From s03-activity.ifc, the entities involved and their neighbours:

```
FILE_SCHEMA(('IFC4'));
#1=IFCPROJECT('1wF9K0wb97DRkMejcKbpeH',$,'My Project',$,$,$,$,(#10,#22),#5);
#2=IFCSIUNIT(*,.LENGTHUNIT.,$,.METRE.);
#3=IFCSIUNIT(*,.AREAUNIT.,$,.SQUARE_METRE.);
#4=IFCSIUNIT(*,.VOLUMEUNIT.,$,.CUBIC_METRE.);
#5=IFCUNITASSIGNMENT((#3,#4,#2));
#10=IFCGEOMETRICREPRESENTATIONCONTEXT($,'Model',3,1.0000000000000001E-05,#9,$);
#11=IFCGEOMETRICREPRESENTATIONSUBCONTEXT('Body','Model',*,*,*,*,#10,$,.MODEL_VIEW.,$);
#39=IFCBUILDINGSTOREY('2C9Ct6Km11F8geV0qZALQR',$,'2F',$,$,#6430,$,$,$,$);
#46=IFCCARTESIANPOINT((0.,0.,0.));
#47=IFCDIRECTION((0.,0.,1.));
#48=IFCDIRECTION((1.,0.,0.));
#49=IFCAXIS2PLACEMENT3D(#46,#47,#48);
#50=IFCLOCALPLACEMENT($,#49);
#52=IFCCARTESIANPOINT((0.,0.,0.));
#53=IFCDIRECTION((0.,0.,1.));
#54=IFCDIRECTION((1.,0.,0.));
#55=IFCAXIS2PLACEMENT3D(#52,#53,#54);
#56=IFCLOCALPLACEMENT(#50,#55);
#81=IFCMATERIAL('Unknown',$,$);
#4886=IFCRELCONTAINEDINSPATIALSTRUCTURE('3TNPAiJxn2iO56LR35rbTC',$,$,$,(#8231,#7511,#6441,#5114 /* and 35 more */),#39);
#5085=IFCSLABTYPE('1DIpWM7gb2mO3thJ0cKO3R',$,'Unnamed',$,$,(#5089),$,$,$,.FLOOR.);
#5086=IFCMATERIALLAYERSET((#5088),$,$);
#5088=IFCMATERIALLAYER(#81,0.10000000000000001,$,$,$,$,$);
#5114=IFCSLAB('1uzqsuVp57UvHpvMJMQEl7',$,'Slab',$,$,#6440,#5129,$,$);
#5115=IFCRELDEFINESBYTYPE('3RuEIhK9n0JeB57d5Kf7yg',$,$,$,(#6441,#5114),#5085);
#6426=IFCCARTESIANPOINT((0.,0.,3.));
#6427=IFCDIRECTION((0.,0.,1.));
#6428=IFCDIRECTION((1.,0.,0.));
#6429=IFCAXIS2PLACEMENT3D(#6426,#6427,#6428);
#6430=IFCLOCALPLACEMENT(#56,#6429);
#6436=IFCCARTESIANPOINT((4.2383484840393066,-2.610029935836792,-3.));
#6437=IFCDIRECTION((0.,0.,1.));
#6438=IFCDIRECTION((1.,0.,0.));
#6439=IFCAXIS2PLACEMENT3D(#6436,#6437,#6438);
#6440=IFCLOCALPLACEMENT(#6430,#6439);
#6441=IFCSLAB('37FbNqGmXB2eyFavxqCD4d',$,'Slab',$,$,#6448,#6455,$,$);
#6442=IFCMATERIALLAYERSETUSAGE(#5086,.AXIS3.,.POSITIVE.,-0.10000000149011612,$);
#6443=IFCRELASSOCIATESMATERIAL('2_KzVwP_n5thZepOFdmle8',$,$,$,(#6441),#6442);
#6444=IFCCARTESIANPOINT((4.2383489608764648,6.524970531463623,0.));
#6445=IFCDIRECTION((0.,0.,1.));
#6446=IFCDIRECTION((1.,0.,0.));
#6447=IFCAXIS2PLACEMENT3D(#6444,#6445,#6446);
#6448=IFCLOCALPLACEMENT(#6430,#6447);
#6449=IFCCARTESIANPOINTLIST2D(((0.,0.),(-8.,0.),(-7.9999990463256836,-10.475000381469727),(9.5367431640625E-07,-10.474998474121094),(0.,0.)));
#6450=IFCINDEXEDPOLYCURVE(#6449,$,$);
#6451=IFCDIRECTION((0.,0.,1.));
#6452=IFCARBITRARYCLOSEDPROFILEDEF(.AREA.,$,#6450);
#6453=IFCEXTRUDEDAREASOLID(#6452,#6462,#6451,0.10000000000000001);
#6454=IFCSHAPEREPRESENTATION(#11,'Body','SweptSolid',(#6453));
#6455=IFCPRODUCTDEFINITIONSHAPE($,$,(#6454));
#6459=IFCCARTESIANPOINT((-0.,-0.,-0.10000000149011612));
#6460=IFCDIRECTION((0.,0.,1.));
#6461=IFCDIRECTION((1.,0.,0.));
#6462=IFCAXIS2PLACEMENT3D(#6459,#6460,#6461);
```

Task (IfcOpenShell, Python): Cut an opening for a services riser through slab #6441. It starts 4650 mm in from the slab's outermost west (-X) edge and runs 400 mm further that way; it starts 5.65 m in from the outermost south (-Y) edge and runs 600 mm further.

```python
import numpy as np
import ifcopenshell
import ifcopenshell.api.feature
import ifcopenshell.api.geometry
import ifcopenshell.api.root
import ifcopenshell.geom
import ifcopenshell.util.placement
import ifcopenshell.util.representation
import ifcopenshell.util.shape
import ifcopenshell.util.unit

model = ifcopenshell.open("s03-activity.ifc")
unit_scale = ifcopenshell.util.unit.calculate_unit_scale(model)
settings = ifcopenshell.geom.settings()


def volume(element):
    """Net volume in cubic metres, openings subtracted."""
    shape = ifcopenshell.geom.create_shape(settings, element)
    return ifcopenshell.util.shape.get_volume(shape.geometry)


slab = model.by_guid("37FbNqGmXB2eyFavxqCD4d")
before = volume(slab)

# Extent in the slab's own axes, in metres. The edges named are its -X and -Y sides.
slab_shape = ifcopenshell.geom.create_shape(settings, slab)
vertices = ifcopenshell.util.shape.get_vertices(slab_shape.geometry)
x_min, y_min, bottom = vertices.min(axis=0)
top = vertices[:, 2].max()

opening = ifcopenshell.api.root.create_entity(model, ifc_class="IfcOpeningElement", name="Services riser opening", predefined_type="OPENING")
context = ifcopenshell.util.representation.get_context(model, "Model", "Body", "MODEL_VIEW")
width, depth = 0.4, 0.6
outline = [(0.0, 0.0), (width, 0.0), (width, depth), (0.0, depth), (0.0, 0.0)]
# Overshoot both faces by 50 mm so the cut is clean.
shape = ifcopenshell.api.geometry.add_slab_representation(
    model, context=context, depth=top - bottom + 0.1, polyline=outline
)
ifcopenshell.api.geometry.assign_representation(model, product=opening, representation=shape)

matrix = ifcopenshell.util.placement.get_local_placement(slab.ObjectPlacement)
matrix[:, 3] = matrix @ np.append(np.array([x_min + 4.65, y_min + 5.65, bottom - 0.05]) / unit_scale, 1.0)
ifcopenshell.api.geometry.edit_object_placement(model, product=opening, matrix=matrix, is_si=False)
ifcopenshell.api.feature.add_feature(model, feature=opening, element=slab)

after = volume(slab)

print(f"slab volume {before:.3f} -> {after:.3f} m3")

model.write("s03-activity_edited.ifc")
```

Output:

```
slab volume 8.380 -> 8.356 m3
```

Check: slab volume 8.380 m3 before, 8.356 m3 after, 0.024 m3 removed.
